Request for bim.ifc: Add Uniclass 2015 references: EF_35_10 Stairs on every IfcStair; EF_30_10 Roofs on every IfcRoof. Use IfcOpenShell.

First a look at what the model holds.

```python
import ifcopenshell

model = ifcopenshell.open("bim.ifc")
print(model.schema)
print("classifications:", [c.Name for c in model.by_type("IfcClassification")])
for ifc_class in ("IfcDoor", "IfcRoof", "IfcStair", "IfcWall", "IfcWindow"):
    print(ifc_class, len(model.by_type(ifc_class)))
```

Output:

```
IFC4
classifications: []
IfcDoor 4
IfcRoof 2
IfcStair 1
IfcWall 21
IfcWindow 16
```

```python
import ifcopenshell
import ifcopenshell.api.classification

model = ifcopenshell.open("bim.ifc")

system = ifcopenshell.api.classification.add_classification(model, classification="Uniclass 2015")

codes = {
    "IfcStair": ("EF_35_10", "Stairs"),
    "IfcRoof": ("EF_30_10", "Roofs"),
}
for ifc_class, (code, name) in codes.items():
    products = model.by_type(ifc_class)
    ifcopenshell.api.classification.add_reference(
        model, products=products, classification=system, identification=code, name=name
    )
    print(code, len(products))

model.write("bim-out.ifc")
```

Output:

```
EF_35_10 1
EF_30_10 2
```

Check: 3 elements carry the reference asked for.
